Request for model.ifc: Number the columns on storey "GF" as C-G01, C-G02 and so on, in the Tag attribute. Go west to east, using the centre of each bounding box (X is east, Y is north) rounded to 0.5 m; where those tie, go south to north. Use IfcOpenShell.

First a look at what the model holds.

```python
import ifcopenshell
import ifcopenshell.util.element
import ifcopenshell.util.placement

model = ifcopenshell.open("model.ifc")
print(model.schema)
storey = next(s for s in model.by_type("IfcBuildingStorey") if s.Name == "GF")
columns = [e for e in ifcopenshell.util.element.get_decomposition(storey) if e.is_a("IfcColumn")]
for e in sorted(columns, key=lambda e: e.id()):
    origin = ifcopenshell.util.placement.get_local_placement(e.ObjectPlacement)[:3, 3]
    print(e.id(), e.Tag, e.Name, origin.round(2) + 0.0, sep=" | ")
```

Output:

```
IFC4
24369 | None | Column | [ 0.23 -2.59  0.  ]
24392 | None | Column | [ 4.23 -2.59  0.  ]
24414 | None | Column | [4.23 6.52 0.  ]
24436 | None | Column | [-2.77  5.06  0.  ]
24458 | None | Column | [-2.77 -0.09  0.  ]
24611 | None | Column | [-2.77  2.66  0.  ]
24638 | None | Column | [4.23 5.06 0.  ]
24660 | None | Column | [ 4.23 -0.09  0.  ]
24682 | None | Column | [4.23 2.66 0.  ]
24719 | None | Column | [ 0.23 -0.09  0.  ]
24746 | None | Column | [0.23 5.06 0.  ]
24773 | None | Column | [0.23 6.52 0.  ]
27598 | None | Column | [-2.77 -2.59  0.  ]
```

```python
import ifcopenshell
import ifcopenshell.geom
import ifcopenshell.util.element
import ifcopenshell.util.shape

model = ifcopenshell.open("model.ifc")
settings = ifcopenshell.geom.settings()
settings.set("use-world-coords", True)


def centre(element):
    shape = ifcopenshell.geom.create_shape(settings, element)
    return ifcopenshell.util.shape.get_bbox_centroid(shape.geometry)


storey = next(s for s in model.by_type("IfcBuildingStorey") if s.Name == "GF")
columns = [e for e in ifcopenshell.util.element.get_decomposition(storey) if e.is_a("IfcColumn")]

# Insertion points can sit at a corner or the storey origin, so sort by the geometry (in metres).
centres = {e: centre(e) for e in columns}
columns.sort(key=lambda e: (round(centres[e][0] / 0.5), centres[e][1]))

for i, e in enumerate(columns, start=1):
    number = f"C-G{i:02d}"
    e.Tag = number
    print(e.id(), number)

model.write("model-out.ifc")
```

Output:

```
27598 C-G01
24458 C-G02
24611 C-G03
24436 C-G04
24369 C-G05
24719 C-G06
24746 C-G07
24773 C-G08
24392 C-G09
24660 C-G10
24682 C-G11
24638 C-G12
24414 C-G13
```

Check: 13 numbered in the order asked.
